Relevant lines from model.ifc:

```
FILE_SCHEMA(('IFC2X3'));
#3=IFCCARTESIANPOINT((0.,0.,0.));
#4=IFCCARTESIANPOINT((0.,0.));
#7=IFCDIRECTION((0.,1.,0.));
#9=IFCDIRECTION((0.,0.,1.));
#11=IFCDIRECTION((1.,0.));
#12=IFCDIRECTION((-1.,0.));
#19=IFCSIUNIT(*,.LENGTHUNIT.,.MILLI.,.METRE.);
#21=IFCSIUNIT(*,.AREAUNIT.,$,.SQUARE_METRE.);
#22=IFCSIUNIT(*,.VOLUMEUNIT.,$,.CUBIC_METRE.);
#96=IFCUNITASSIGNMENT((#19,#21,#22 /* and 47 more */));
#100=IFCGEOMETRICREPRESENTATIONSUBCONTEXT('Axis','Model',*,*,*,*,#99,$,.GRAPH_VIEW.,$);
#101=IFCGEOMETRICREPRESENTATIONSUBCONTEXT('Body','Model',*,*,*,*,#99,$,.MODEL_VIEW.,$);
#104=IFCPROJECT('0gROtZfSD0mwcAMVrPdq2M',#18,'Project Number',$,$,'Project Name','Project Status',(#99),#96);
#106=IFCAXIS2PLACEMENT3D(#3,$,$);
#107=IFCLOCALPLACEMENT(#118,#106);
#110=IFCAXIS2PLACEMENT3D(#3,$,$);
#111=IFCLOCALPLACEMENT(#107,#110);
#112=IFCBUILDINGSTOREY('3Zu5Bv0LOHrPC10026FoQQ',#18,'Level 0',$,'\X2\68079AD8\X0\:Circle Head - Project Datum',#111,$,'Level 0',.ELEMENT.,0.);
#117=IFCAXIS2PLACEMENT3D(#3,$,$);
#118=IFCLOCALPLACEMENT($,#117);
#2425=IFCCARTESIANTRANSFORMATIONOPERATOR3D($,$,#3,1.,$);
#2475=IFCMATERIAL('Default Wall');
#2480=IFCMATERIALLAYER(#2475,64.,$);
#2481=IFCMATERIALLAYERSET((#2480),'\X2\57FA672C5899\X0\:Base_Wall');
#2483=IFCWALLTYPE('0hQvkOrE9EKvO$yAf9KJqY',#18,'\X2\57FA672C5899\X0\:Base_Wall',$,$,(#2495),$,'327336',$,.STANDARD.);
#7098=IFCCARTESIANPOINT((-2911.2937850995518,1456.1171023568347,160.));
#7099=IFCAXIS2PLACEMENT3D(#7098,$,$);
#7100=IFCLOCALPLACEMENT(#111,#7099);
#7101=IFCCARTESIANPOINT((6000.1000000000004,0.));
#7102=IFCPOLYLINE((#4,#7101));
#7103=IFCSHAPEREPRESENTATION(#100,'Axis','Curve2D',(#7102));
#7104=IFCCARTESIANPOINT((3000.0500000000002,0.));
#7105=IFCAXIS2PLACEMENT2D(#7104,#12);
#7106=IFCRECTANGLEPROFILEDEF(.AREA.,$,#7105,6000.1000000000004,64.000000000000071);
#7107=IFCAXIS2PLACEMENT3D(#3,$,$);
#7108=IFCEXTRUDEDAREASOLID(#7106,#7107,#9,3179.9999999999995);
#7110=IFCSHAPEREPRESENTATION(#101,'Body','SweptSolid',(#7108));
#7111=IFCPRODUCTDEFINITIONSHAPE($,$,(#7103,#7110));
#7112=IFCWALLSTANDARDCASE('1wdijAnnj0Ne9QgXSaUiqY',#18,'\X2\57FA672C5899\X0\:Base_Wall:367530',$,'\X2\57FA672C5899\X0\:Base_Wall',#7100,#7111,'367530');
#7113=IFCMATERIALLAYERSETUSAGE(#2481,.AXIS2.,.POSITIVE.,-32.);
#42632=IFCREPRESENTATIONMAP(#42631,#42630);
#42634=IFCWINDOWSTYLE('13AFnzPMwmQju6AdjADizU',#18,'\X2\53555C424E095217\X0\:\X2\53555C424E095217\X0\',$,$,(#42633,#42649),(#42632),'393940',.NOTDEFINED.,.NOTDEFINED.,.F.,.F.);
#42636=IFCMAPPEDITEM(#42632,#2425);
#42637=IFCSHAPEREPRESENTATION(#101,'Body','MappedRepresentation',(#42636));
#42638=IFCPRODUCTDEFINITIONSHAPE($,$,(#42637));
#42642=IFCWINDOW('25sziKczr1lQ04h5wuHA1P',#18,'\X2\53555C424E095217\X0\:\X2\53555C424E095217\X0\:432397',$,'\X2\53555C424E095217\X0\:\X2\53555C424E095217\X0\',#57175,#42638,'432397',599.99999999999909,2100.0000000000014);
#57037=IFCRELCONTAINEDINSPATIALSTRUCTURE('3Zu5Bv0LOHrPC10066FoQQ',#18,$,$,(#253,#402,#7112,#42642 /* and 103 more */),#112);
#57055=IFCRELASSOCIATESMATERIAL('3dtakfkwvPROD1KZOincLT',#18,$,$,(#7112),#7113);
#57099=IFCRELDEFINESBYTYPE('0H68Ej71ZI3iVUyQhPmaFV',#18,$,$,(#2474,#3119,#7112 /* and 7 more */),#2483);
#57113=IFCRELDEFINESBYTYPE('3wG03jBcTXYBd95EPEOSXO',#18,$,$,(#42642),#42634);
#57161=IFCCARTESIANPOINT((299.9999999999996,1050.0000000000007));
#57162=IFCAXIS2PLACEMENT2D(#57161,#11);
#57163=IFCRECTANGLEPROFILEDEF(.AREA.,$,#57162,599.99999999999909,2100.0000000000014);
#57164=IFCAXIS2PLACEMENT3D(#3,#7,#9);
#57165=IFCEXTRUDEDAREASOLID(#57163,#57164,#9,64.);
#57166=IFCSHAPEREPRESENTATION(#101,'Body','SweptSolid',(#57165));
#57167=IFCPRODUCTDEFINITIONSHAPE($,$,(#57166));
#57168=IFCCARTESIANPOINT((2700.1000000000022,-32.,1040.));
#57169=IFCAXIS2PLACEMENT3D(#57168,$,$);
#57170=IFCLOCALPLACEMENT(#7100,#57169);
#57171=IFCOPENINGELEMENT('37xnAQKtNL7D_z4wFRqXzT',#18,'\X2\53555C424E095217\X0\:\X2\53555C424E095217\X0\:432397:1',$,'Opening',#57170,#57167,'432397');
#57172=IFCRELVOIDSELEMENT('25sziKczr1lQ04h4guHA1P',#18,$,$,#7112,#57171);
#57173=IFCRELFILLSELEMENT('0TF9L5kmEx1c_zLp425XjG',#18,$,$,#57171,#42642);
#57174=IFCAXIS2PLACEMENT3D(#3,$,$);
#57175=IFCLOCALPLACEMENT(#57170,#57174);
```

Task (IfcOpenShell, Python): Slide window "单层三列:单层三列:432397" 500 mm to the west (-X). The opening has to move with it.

```python
import ifcopenshell
import ifcopenshell.api.geometry
import ifcopenshell.util.placement

model = ifcopenshell.open("model.ifc")

window = model.by_id(42642)
opening = window.FillsVoids[0].RelatingOpeningElement
wall = opening.VoidsElements[0].RelatingBuildingElement

wall_matrix = ifcopenshell.util.placement.get_local_placement(wall.ObjectPlacement)
shift = wall_matrix[:3, 0] * -500.0
before = ifcopenshell.util.placement.get_local_placement(window.ObjectPlacement)[:3, 3].copy()

# The window is placed relative to its opening, so it follows when the opening moves.
matrix = ifcopenshell.util.placement.get_local_placement(opening.ObjectPlacement)
matrix[:3, 3] += shift
ifcopenshell.api.geometry.edit_object_placement(
    model, product=opening, matrix=matrix, is_si=False, should_transform_children=True
)

after = ifcopenshell.util.placement.get_local_placement(window.ObjectPlacement)[:3, 3]
print("window moved by", (after - before).round(3) + 0.0)

model.write("model_v2.ifc")
```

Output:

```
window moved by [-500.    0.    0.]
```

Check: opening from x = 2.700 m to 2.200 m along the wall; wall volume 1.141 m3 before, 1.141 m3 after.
